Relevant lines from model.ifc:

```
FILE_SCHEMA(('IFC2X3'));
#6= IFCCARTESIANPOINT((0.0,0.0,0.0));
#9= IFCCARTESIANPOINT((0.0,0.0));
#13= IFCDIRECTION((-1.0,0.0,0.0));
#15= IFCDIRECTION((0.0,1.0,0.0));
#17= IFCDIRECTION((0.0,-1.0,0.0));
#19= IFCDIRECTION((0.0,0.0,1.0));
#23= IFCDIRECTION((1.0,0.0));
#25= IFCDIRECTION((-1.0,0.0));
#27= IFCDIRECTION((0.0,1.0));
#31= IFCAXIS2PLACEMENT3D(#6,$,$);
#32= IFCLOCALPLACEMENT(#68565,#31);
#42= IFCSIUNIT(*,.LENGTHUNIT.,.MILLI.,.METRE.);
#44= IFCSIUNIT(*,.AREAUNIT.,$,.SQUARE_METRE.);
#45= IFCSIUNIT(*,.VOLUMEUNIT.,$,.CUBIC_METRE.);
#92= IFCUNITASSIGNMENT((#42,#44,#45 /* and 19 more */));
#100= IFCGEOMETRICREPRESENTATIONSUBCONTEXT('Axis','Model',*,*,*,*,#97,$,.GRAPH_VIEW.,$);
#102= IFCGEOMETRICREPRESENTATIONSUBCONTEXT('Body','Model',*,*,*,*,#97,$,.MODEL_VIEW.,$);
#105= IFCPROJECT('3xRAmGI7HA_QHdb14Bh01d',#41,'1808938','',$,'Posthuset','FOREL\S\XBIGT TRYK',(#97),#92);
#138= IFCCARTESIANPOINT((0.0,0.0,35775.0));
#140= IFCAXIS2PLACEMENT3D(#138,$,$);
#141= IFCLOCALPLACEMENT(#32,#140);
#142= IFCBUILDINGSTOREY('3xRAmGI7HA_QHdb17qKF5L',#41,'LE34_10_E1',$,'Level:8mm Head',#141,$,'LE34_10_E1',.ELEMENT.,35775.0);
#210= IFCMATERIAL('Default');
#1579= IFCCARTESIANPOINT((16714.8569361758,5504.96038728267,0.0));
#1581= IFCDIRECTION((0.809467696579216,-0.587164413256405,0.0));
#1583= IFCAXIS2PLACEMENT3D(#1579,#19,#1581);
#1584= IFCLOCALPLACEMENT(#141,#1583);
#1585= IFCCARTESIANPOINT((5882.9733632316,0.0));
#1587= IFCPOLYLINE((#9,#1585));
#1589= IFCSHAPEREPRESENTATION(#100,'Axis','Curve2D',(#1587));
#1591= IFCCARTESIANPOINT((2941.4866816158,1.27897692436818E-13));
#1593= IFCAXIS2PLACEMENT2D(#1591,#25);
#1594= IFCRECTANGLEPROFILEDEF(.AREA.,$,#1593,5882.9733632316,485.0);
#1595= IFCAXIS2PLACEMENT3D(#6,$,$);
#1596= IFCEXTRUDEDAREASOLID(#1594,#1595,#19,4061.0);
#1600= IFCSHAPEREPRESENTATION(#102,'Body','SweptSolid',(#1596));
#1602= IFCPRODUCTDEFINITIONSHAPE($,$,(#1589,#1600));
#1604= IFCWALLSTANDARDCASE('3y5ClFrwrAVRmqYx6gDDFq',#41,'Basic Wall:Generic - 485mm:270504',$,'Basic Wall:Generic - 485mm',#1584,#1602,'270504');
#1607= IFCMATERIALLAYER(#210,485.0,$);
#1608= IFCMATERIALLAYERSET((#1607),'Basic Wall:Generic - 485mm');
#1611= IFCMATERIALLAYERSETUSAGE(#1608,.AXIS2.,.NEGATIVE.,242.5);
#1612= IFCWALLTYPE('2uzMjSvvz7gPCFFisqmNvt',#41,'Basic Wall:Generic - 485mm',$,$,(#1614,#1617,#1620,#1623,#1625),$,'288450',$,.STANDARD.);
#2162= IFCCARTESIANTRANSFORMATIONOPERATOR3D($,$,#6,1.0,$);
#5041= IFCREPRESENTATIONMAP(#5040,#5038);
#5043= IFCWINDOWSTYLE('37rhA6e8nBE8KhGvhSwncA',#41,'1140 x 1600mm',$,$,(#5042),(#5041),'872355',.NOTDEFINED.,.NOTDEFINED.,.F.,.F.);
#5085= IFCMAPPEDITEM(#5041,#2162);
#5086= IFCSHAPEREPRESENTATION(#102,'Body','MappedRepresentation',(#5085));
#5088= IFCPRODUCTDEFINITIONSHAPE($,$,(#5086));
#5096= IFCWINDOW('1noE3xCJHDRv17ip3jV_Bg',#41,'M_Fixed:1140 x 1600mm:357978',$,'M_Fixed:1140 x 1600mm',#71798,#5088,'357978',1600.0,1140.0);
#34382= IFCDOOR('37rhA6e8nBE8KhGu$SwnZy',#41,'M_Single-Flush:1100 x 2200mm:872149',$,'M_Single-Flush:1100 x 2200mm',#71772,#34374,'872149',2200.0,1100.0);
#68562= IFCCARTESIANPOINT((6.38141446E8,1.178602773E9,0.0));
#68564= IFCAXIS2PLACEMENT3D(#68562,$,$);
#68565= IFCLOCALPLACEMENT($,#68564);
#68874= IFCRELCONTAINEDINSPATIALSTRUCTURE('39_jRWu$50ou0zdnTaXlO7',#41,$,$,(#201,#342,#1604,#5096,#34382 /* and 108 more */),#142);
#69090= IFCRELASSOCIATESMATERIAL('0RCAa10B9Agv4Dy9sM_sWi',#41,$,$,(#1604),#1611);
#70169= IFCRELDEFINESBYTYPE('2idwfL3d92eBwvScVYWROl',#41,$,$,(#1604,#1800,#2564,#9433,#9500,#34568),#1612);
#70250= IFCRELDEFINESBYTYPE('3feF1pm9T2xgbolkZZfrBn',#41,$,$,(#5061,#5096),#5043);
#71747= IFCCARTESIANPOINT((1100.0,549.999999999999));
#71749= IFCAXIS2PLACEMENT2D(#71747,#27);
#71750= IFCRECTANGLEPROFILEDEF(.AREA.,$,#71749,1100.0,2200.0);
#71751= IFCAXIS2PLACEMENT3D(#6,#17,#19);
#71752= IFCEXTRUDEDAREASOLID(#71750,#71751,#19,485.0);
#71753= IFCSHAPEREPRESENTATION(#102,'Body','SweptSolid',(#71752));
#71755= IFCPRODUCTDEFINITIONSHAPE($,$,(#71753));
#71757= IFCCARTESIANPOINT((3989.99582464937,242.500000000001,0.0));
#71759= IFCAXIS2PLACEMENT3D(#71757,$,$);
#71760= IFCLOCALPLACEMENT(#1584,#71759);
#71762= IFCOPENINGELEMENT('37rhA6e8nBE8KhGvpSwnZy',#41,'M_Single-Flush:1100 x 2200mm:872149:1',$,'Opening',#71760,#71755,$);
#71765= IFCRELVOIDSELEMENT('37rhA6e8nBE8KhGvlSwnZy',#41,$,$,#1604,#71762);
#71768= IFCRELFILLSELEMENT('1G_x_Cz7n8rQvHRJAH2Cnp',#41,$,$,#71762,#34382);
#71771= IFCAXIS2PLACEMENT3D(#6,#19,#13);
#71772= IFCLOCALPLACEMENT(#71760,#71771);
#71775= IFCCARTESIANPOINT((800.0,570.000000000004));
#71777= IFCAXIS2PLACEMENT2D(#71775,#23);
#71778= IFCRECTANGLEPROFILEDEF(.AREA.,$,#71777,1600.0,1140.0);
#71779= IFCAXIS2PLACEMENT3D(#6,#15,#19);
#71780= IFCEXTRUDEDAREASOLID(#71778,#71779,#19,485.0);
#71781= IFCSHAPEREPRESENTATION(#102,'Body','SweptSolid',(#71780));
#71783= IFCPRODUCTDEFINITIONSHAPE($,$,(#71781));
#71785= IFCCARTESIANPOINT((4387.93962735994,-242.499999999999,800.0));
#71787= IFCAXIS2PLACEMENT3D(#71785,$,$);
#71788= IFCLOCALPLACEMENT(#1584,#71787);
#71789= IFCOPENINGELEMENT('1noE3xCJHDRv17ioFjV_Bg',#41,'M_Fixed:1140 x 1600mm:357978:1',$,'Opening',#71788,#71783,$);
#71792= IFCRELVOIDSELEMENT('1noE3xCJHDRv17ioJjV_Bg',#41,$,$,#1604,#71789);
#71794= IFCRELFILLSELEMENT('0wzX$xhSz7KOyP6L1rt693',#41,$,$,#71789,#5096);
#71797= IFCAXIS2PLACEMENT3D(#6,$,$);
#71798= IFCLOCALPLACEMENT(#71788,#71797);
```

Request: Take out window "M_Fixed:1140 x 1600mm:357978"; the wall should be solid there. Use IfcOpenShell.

```python
import ifcopenshell
import ifcopenshell.api.feature
import ifcopenshell.api.root
import ifcopenshell.geom
import ifcopenshell.util.shape

model = ifcopenshell.open("model.ifc")
settings = ifcopenshell.geom.settings()


def volume(element):
    """Net volume in cubic metres, openings subtracted."""
    shape = ifcopenshell.geom.create_shape(settings, element)
    return ifcopenshell.util.shape.get_volume(shape.geometry)


window = model.by_guid("1noE3xCJHDRv17ip3jV_Bg")
opening = window.FillsVoids[0].RelatingOpeningElement
wall = opening.VoidsElements[0].RelatingBuildingElement
before = volume(wall)

ifcopenshell.api.root.remove_product(model, product=window)
ifcopenshell.api.feature.remove_feature(model, feature=opening)

after = volume(wall)

print(f"wall volume {before:.3f} -> {after:.3f} m3")

model.write("model_edited.ifc")
```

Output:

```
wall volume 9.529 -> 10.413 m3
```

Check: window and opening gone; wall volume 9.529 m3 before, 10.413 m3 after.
